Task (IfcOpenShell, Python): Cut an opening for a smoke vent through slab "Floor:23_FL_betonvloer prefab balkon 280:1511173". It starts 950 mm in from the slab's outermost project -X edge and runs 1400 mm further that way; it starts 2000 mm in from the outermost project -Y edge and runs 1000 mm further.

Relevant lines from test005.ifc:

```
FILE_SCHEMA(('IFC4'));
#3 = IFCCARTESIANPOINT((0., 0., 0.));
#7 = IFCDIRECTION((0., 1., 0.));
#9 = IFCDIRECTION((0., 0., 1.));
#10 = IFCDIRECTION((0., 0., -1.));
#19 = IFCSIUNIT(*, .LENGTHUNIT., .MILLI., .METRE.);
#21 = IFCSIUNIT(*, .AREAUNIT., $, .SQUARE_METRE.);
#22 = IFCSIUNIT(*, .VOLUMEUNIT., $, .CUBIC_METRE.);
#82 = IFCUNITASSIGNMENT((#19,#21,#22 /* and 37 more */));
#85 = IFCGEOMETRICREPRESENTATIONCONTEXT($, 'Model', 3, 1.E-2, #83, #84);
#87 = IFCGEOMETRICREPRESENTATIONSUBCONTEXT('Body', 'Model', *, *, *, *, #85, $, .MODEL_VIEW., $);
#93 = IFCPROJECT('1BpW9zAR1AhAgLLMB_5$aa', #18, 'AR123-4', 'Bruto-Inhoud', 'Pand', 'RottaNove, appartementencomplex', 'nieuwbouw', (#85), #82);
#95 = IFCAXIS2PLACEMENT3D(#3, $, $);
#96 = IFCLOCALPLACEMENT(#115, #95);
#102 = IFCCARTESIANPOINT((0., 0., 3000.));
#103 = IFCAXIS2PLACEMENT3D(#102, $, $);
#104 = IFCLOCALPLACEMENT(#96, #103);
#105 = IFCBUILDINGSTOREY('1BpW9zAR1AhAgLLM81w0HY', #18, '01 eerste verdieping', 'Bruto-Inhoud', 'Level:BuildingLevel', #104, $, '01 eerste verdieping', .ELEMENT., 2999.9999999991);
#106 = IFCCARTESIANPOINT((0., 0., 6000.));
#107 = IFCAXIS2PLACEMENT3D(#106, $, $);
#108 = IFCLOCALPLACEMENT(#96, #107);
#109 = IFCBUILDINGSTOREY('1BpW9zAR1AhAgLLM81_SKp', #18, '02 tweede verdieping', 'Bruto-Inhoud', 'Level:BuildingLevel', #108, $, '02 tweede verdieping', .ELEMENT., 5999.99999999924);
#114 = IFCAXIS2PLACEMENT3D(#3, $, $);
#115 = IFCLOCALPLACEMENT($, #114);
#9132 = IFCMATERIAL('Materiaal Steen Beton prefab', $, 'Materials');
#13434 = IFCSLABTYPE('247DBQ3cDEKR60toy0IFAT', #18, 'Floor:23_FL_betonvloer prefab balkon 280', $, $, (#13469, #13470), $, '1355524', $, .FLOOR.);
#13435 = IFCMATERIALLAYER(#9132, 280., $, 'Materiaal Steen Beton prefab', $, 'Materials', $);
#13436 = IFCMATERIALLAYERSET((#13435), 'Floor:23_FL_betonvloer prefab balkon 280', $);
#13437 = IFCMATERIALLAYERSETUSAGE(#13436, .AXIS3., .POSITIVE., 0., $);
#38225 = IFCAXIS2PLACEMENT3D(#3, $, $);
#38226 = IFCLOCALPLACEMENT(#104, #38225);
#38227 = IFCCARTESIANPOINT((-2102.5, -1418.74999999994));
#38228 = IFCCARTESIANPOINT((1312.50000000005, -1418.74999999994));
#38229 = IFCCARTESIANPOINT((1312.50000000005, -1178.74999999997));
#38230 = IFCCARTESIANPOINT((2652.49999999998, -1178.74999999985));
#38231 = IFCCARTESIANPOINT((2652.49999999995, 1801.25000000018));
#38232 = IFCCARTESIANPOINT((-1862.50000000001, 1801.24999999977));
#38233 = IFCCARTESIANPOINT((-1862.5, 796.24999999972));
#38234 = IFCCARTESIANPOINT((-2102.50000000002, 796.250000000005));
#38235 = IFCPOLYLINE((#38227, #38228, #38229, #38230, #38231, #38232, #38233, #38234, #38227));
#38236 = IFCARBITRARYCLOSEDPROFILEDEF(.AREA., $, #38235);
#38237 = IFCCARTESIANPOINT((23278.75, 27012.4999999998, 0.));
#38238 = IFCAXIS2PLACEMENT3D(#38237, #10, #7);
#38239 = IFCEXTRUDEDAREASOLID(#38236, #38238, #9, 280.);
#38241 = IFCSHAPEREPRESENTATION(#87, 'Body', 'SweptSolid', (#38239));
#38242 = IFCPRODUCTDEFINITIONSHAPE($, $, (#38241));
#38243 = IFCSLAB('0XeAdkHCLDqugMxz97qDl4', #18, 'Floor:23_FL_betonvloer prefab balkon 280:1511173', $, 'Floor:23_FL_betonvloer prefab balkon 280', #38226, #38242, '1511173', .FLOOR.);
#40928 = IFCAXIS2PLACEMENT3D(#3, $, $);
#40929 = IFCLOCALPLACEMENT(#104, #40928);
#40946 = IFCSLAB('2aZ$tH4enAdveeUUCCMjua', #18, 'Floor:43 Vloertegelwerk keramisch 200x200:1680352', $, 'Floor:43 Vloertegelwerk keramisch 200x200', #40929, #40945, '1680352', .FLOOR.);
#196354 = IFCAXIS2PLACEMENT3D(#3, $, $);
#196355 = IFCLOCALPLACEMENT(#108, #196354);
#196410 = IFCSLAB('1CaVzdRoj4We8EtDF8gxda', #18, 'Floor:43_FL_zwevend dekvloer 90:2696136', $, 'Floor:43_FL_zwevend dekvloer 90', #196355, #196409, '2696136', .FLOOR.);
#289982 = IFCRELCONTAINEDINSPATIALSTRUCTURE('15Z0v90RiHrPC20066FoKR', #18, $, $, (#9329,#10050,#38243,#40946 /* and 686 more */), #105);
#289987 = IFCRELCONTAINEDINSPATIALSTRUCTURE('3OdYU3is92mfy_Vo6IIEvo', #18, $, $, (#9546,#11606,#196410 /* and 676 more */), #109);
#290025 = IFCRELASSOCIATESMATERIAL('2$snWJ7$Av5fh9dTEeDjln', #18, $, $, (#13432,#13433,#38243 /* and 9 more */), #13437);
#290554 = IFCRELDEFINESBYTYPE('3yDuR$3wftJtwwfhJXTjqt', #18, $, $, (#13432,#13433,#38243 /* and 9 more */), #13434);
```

```python
import numpy as np
import ifcopenshell
import ifcopenshell.api.feature
import ifcopenshell.api.geometry
import ifcopenshell.api.root
import ifcopenshell.geom
import ifcopenshell.util.placement
import ifcopenshell.util.representation
import ifcopenshell.util.shape
import ifcopenshell.util.unit

model = ifcopenshell.open("test005.ifc")
unit_scale = ifcopenshell.util.unit.calculate_unit_scale(model)
settings = ifcopenshell.geom.settings()


def volume(element):
    """Net volume in cubic metres, openings subtracted."""
    shape = ifcopenshell.geom.create_shape(settings, element)
    return ifcopenshell.util.shape.get_volume(shape.geometry)


slab = model.by_id(38243)
before = volume(slab)

# Extent in the slab's own axes, in metres. The edges named are its -X and -Y sides.
slab_shape = ifcopenshell.geom.create_shape(settings, slab)
vertices = ifcopenshell.util.shape.get_vertices(slab_shape.geometry)
x_min, y_min, bottom = vertices.min(axis=0)
top = vertices[:, 2].max()

opening = ifcopenshell.api.root.create_entity(model, ifc_class="IfcOpeningElement", name="Smoke vent opening", predefined_type="OPENING")
context = ifcopenshell.util.representation.get_context(model, "Model", "Body", "MODEL_VIEW")
width, depth = 1.4, 1
outline = [(0.0, 0.0), (width, 0.0), (width, depth), (0.0, depth), (0.0, 0.0)]
# Overshoot both faces by 50 mm so the cut is clean.
shape = ifcopenshell.api.geometry.add_slab_representation(
    model, context=context, depth=top - bottom + 0.1, polyline=outline
)
ifcopenshell.api.geometry.assign_representation(model, product=opening, representation=shape)

matrix = ifcopenshell.util.placement.get_local_placement(slab.ObjectPlacement)
matrix[:, 3] = matrix @ np.append(np.array([x_min + 0.95, y_min + 2, bottom - 0.05]) / unit_scale, 1.0)
ifcopenshell.api.geometry.edit_object_placement(model, product=opening, matrix=matrix, is_si=False)
ifcopenshell.api.feature.add_feature(model, feature=opening, element=slab)

after = volume(slab)

print(f"slab volume {before:.3f} -> {after:.3f} m3")

model.write("test005_updated.ifc")
```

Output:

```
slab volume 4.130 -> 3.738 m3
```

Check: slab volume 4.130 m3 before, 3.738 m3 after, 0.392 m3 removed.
